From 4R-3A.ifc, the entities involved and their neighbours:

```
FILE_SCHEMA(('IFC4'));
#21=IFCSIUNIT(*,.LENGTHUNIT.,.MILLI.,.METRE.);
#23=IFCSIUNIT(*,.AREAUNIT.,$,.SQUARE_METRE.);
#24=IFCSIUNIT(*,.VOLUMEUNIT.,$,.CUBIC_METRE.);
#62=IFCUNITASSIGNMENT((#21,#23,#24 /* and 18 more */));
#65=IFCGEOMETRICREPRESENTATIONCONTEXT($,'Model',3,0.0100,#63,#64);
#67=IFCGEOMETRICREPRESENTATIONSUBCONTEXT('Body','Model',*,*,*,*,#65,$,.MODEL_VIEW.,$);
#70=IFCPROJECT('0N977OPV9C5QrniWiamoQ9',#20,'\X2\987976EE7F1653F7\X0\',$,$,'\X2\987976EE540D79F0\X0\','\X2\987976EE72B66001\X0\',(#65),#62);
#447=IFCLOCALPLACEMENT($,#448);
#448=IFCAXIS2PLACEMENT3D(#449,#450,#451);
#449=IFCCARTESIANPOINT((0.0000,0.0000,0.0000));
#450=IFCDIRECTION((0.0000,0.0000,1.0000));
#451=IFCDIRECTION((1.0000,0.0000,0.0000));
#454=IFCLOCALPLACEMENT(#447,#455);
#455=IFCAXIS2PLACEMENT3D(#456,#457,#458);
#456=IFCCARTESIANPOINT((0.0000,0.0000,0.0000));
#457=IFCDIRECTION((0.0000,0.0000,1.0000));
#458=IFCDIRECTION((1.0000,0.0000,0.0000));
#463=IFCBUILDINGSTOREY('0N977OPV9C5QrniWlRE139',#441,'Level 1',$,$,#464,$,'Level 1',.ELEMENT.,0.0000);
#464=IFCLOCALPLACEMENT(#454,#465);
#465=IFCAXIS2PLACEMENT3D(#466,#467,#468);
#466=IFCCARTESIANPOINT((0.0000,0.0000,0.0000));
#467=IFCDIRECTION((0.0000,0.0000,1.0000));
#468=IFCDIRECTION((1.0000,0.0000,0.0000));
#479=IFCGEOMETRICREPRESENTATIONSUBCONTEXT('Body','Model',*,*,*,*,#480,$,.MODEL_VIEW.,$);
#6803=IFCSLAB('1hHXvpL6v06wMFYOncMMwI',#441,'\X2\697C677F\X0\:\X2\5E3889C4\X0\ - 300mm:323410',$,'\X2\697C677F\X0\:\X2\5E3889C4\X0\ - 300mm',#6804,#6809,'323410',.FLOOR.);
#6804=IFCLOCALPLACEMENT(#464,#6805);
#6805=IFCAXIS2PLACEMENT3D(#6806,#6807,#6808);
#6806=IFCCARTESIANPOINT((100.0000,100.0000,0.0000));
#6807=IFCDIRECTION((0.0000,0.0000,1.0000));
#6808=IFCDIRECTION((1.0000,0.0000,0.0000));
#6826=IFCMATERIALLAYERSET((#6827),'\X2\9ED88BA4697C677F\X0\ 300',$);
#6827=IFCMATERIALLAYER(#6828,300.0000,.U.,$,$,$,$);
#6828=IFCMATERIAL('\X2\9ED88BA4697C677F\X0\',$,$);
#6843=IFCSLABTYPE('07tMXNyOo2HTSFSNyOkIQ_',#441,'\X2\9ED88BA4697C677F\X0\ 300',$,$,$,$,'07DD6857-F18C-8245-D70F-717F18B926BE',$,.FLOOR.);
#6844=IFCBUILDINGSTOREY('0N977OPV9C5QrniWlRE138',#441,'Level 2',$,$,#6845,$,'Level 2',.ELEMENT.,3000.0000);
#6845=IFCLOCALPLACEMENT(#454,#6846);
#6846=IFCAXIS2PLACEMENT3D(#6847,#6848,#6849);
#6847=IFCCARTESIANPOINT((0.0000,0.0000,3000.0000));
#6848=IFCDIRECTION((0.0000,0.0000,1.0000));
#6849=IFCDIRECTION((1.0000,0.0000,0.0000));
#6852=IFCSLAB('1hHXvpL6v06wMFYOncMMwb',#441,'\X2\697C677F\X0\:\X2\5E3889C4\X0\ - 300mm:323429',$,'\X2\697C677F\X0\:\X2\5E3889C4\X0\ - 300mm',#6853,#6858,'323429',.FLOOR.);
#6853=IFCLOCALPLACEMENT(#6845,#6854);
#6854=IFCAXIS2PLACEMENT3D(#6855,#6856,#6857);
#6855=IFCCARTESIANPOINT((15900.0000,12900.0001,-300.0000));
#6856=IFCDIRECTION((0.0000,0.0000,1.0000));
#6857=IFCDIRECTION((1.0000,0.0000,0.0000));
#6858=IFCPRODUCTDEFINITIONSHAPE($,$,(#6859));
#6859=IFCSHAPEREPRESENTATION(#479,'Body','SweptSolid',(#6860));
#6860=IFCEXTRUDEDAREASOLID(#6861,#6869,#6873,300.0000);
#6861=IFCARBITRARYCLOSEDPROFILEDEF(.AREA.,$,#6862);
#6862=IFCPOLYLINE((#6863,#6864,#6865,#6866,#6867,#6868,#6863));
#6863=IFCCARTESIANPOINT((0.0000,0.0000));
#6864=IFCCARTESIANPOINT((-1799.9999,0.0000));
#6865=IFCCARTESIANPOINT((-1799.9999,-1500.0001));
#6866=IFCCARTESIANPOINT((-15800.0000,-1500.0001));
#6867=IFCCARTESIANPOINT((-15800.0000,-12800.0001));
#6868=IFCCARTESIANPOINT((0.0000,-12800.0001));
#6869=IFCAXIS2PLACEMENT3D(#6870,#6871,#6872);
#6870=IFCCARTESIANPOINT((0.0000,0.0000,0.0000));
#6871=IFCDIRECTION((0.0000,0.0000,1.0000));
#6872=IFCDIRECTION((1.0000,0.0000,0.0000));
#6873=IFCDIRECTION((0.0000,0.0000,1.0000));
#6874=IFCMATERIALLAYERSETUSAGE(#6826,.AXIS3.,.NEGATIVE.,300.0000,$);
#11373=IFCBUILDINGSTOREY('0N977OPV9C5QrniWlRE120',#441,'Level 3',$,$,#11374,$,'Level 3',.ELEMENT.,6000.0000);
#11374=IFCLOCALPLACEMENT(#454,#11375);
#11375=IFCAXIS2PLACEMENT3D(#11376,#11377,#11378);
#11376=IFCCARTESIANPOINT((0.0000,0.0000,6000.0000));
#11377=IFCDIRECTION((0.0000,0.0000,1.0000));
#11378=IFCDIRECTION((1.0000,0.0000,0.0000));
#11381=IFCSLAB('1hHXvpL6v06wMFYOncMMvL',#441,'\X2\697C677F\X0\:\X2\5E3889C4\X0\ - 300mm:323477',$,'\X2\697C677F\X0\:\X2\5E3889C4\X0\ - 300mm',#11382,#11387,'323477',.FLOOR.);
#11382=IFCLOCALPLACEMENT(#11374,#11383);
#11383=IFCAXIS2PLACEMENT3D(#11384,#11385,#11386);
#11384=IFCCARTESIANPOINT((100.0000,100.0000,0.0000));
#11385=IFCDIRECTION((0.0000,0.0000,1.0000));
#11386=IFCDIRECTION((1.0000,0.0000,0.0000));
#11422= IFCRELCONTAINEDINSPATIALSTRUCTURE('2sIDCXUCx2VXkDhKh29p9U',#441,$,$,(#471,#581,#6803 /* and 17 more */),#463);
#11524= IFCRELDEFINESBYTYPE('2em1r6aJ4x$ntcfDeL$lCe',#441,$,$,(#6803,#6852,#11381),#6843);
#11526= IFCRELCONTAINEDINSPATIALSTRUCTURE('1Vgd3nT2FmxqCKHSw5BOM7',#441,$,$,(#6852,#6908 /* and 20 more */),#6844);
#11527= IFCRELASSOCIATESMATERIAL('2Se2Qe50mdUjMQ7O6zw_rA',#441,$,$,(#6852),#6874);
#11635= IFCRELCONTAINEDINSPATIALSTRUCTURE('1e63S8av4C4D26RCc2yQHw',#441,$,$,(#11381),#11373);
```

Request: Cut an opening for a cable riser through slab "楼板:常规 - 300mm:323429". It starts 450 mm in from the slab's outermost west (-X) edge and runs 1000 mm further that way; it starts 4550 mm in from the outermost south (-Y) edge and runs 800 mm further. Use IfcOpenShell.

```python
import numpy as np
import ifcopenshell
import ifcopenshell.api.feature
import ifcopenshell.api.geometry
import ifcopenshell.api.root
import ifcopenshell.geom
import ifcopenshell.util.placement
import ifcopenshell.util.representation
import ifcopenshell.util.shape
import ifcopenshell.util.unit

model = ifcopenshell.open("4R-3A.ifc")
unit_scale = ifcopenshell.util.unit.calculate_unit_scale(model)
settings = ifcopenshell.geom.settings()


def volume(element):
    """Net volume in cubic metres, openings subtracted."""
    shape = ifcopenshell.geom.create_shape(settings, element)
    return ifcopenshell.util.shape.get_volume(shape.geometry)


slab = model.by_guid("1hHXvpL6v06wMFYOncMMwb")
before = volume(slab)

# Extent in the slab's own axes, in metres. The edges named are its -X and -Y sides.
slab_shape = ifcopenshell.geom.create_shape(settings, slab)
vertices = ifcopenshell.util.shape.get_vertices(slab_shape.geometry)
x_min, y_min, bottom = vertices.min(axis=0)
top = vertices[:, 2].max()

opening = ifcopenshell.api.root.create_entity(model, ifc_class="IfcOpeningElement", name="Cable riser opening", predefined_type="OPENING")
context = ifcopenshell.util.representation.get_context(model, "Model", "Body", "MODEL_VIEW")
width, depth = 1, 0.8
outline = [(0.0, 0.0), (width, 0.0), (width, depth), (0.0, depth), (0.0, 0.0)]
# Overshoot both faces by 50 mm so the cut is clean.
shape = ifcopenshell.api.geometry.add_slab_representation(
    model, context=context, depth=top - bottom + 0.1, polyline=outline
)
ifcopenshell.api.geometry.assign_representation(model, product=opening, representation=shape)

matrix = ifcopenshell.util.placement.get_local_placement(slab.ObjectPlacement)
matrix[:, 3] = matrix @ np.append(np.array([x_min + 0.45, y_min + 4.55, bottom - 0.05]) / unit_scale, 1.0)
ifcopenshell.api.geometry.edit_object_placement(model, product=opening, matrix=matrix, is_si=False)
ifcopenshell.api.feature.add_feature(model, feature=opening, element=slab)

after = volume(slab)

print(f"slab volume {before:.3f} -> {after:.3f} m3")

model.write("4R-3A_edited.ifc")
```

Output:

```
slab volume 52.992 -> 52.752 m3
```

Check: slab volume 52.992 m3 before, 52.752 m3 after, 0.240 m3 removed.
